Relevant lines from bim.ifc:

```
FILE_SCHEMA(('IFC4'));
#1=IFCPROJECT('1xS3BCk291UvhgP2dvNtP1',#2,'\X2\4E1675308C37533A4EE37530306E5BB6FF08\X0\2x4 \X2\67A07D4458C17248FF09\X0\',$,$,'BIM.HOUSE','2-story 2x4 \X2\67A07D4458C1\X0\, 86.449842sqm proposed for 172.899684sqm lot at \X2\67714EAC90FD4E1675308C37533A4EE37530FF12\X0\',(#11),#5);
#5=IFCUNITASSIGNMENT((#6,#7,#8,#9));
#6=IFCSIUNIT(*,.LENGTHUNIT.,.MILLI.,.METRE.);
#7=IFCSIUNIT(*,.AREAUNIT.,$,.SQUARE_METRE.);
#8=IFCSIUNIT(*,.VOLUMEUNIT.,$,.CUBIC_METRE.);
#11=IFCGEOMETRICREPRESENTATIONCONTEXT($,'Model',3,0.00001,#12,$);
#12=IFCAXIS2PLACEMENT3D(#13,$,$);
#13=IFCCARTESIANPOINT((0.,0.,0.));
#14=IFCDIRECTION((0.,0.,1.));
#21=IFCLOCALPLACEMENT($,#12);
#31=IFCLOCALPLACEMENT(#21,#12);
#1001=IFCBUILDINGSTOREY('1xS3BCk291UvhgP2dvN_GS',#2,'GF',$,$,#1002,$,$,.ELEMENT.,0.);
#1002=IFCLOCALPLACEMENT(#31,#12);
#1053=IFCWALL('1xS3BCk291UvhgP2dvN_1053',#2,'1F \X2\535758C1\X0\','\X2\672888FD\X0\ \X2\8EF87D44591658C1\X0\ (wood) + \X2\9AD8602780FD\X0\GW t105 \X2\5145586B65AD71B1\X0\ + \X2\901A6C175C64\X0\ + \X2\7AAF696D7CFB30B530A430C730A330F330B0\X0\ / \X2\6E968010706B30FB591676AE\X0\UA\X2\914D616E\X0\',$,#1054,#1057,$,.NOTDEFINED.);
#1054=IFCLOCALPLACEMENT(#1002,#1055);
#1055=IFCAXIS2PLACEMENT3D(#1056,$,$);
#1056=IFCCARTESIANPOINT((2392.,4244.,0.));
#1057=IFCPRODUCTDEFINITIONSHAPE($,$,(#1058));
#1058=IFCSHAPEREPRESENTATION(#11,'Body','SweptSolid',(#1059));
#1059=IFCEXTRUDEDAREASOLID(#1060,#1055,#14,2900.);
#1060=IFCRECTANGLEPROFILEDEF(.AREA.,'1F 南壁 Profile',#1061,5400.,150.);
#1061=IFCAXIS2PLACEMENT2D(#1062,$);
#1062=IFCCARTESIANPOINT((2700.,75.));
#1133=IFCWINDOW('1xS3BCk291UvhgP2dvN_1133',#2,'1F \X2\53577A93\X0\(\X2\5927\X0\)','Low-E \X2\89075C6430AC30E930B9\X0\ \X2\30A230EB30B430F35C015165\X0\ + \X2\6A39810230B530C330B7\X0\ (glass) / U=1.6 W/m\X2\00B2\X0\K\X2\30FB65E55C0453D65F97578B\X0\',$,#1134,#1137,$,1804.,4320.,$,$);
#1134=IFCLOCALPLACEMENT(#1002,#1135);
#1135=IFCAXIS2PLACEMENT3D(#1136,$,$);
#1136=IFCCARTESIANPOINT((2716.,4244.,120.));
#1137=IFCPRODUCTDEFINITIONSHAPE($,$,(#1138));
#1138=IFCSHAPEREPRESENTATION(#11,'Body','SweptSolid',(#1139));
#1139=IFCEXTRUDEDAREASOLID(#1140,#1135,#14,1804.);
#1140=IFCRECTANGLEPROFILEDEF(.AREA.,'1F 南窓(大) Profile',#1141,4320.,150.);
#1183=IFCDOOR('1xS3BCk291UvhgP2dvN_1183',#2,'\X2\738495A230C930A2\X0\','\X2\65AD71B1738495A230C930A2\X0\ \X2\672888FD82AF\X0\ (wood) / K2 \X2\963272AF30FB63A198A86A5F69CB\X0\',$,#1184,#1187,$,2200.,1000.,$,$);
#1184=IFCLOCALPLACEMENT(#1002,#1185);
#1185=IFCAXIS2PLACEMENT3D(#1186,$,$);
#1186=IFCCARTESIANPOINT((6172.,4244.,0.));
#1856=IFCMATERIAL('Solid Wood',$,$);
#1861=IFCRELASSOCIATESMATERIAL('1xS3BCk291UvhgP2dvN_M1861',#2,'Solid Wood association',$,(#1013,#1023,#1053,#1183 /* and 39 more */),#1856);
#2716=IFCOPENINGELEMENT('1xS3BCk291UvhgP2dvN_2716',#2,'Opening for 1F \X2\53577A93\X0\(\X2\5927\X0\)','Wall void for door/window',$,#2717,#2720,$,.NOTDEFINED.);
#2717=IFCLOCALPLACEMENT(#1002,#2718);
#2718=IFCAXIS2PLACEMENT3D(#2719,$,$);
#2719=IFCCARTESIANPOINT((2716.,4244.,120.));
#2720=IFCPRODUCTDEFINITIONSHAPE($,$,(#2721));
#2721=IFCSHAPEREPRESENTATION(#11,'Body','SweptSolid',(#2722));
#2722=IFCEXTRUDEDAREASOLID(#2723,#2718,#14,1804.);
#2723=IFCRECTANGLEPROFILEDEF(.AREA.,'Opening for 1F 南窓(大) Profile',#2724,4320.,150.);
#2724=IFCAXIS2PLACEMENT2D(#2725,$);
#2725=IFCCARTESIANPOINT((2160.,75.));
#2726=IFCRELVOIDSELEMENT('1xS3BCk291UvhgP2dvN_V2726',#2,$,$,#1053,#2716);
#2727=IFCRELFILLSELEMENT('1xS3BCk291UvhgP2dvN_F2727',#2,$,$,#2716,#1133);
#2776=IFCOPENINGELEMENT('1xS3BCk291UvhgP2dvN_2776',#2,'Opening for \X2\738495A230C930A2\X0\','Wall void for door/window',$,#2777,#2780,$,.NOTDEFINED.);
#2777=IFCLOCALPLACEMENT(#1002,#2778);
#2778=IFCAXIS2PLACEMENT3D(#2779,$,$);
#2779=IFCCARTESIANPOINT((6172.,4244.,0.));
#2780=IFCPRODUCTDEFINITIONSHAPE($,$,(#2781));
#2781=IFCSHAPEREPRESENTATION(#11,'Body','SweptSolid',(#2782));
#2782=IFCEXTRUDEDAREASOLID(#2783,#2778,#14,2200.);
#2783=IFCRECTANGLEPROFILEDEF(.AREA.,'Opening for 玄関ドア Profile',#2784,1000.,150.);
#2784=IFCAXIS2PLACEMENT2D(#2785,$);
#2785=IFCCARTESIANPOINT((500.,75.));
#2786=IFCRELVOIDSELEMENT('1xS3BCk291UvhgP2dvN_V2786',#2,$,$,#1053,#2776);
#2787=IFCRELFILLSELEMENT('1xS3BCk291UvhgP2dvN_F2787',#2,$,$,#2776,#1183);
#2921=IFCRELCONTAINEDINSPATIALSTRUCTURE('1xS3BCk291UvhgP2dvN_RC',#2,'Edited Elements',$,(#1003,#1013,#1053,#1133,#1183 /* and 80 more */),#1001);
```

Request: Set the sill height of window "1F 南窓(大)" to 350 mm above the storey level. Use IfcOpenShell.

```python
import numpy as np
import ifcopenshell
import ifcopenshell.api.geometry
import ifcopenshell.geom
import ifcopenshell.util.element
import ifcopenshell.util.placement
import ifcopenshell.util.shape
import ifcopenshell.util.unit

model = ifcopenshell.open("bim.ifc")
unit_scale = ifcopenshell.util.unit.calculate_unit_scale(model)

window = model.by_guid("1xS3BCk291UvhgP2dvN_1133")
opening = window.FillsVoids[0].RelatingOpeningElement
storey = ifcopenshell.util.element.get_container(window, ifc_class="IfcBuildingStorey")
level = ifcopenshell.util.placement.get_local_placement(storey.ObjectPlacement)[2, 3]

# The opening's origin need not be at the sill, so measure its lowest point.
shape = ifcopenshell.geom.create_shape(ifcopenshell.geom.settings(), opening)
bottom = ifcopenshell.util.shape.get_shape_bottom_elevation(shape, shape.geometry) / unit_scale
dz = level + 0.35 / unit_scale - bottom

shift = np.array([0.0, 0.0, dz])
# The window is not placed relative to its opening, so move both.
for product in (opening, window):
    matrix = ifcopenshell.util.placement.get_local_placement(product.ObjectPlacement)
    matrix[:3, 3] += shift
    ifcopenshell.api.geometry.edit_object_placement(model, product=product, matrix=matrix, is_si=False)

print(f"moved by {dz * unit_scale:+.3f} m")

model.write("bim_rev.ifc")
```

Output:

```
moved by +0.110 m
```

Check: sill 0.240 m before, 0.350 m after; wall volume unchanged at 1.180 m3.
